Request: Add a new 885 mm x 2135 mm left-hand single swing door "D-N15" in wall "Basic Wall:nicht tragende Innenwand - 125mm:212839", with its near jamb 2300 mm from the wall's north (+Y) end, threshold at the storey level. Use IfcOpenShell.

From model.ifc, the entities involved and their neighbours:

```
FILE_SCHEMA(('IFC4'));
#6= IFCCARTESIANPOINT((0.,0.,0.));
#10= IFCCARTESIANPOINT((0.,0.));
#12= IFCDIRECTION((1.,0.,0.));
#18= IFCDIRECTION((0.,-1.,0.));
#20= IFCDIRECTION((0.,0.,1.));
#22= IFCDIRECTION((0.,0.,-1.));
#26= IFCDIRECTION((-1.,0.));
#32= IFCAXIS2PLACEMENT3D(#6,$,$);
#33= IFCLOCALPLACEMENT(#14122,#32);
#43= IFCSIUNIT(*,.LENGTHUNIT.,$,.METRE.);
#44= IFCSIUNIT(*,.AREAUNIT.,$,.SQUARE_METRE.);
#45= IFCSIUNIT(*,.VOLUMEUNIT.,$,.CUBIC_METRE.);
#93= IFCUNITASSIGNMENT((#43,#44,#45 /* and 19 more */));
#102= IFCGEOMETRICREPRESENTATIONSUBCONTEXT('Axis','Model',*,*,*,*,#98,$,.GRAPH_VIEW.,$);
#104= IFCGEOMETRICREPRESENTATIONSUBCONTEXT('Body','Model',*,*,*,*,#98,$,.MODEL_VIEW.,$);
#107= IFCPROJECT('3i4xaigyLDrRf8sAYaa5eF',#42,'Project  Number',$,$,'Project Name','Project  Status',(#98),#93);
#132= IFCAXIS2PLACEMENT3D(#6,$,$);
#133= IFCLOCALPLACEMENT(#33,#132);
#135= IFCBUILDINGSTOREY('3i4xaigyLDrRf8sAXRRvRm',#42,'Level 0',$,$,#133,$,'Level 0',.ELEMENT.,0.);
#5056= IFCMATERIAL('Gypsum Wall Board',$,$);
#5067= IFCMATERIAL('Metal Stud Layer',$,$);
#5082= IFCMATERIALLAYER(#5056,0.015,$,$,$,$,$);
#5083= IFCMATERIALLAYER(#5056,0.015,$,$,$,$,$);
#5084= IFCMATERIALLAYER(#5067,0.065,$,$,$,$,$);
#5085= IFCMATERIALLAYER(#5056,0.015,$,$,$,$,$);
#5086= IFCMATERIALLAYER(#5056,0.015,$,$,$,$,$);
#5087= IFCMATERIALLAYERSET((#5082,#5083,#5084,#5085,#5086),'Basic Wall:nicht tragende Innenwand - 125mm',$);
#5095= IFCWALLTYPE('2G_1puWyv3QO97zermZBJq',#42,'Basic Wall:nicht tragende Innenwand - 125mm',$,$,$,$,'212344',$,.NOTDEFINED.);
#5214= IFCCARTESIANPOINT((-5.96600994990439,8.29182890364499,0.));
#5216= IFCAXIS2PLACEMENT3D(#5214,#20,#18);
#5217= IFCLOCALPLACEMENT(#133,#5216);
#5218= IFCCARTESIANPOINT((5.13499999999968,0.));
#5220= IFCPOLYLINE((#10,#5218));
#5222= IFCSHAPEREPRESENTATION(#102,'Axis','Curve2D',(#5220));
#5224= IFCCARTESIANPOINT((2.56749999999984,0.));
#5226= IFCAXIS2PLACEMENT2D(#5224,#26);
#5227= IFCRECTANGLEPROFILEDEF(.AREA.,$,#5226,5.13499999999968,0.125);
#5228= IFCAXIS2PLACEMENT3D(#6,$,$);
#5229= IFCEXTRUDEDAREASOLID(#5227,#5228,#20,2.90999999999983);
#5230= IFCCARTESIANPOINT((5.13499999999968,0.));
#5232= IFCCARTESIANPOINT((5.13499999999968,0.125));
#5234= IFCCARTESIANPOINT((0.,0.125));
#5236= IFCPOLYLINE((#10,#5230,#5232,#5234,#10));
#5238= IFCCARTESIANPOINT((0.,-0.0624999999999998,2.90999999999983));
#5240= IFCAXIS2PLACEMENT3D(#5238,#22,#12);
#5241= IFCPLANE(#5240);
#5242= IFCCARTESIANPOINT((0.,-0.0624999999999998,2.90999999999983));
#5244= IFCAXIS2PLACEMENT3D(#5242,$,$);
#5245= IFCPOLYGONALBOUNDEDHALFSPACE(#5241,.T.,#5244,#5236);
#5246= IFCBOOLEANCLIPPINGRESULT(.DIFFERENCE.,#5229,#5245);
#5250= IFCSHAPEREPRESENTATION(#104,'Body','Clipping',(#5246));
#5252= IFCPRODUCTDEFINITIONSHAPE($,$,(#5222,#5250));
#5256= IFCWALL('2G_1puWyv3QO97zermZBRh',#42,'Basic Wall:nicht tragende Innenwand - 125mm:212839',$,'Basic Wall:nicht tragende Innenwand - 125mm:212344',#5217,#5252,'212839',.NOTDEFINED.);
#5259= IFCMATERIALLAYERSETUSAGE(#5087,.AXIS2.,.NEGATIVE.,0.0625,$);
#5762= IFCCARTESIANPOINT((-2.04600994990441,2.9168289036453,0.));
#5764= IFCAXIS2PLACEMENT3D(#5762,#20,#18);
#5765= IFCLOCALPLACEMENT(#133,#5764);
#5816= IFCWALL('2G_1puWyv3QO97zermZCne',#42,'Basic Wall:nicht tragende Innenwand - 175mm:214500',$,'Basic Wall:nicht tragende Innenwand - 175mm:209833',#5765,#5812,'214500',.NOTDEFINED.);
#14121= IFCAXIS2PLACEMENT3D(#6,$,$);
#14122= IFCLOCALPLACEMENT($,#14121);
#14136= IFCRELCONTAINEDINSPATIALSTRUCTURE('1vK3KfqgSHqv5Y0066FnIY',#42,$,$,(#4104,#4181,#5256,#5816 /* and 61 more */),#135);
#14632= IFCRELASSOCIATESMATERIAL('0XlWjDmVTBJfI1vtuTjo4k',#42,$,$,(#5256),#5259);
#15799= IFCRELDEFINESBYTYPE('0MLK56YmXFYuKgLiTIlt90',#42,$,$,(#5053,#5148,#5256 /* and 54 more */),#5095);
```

```python
import numpy as np
import ifcopenshell
import ifcopenshell.api.feature
import ifcopenshell.api.geometry
import ifcopenshell.api.root
import ifcopenshell.api.spatial
import ifcopenshell.geom
import ifcopenshell.util.element
import ifcopenshell.util.placement
import ifcopenshell.util.representation
import ifcopenshell.util.shape
import ifcopenshell.util.unit

model = ifcopenshell.open("model.ifc")
unit_scale = ifcopenshell.util.unit.calculate_unit_scale(model)
settings = ifcopenshell.geom.settings()


def volume(element):
    """Net volume in cubic metres, openings subtracted."""
    shape = ifcopenshell.geom.create_shape(settings, element)
    return ifcopenshell.util.shape.get_volume(shape.geometry)


wall = model.by_guid("2G_1puWyv3QO97zermZBRh")
storey = ifcopenshell.util.element.get_container(wall, ifc_class="IfcBuildingStorey")
context = ifcopenshell.util.representation.get_context(model, "Model", "Body", "MODEL_VIEW")
before = volume(wall)

width, height, from_end, sill = 0.885, 2.135, 2.3, 0.0  # metres

# The wall runs along its own X axis, and the end named is its -X end.
wall_shape = ifcopenshell.geom.create_shape(settings, wall)
x, y, z = ifcopenshell.util.shape.get_vertices(wall_shape.geometry).T
start = x.min() + from_end
face, thickness = float(y.min()), float(y.max() - y.min())
wall_matrix = ifcopenshell.util.placement.get_local_placement(wall.ObjectPlacement)
level = ifcopenshell.util.placement.get_local_placement(storey.ObjectPlacement)[2, 3]


def in_wall(x, y):
    """Placement at x, y metres in the wall's axes, at sill height."""
    matrix = wall_matrix.copy()
    matrix[:, 3] = wall_matrix @ np.array([x / unit_scale, y / unit_scale, 0.0, 1.0])
    matrix[2, 3] = level + sill / unit_scale
    return matrix


# Opening: a box that overshoots both wall faces by 50 mm.
opening = ifcopenshell.api.root.create_entity(model, ifc_class="IfcOpeningElement", predefined_type="OPENING")
box = ifcopenshell.api.geometry.add_wall_representation(
    model, context=context, length=width, height=height, thickness=thickness + 0.1
)
ifcopenshell.api.geometry.assign_representation(model, product=opening, representation=box)
ifcopenshell.api.geometry.edit_object_placement(model, product=opening, matrix=in_wall(start, face - 0.05), is_si=False)
ifcopenshell.api.feature.add_feature(model, feature=opening, element=wall)

door = ifcopenshell.api.root.create_entity(model, ifc_class="IfcDoor", name="D-N15", predefined_type="DOOR")
door.OverallWidth, door.OverallHeight = width / unit_scale, height / unit_scale
door.OperationType = "SINGLE_SWING_LEFT"
body = ifcopenshell.api.geometry.add_door_representation(
    model,
    context=context,
    overall_width=door.OverallWidth,
    overall_height=door.OverallHeight,
    operation_type="SINGLE_SWING_LEFT",
    lining_properties={"LiningDepth": thickness / unit_scale, "ThresholdDepth": thickness / unit_scale},
)
ifcopenshell.api.geometry.assign_representation(model, product=door, representation=body)
ifcopenshell.api.spatial.assign_container(model, products=[door], relating_structure=storey)
ifcopenshell.api.feature.add_filling(model, opening=opening, element=door)

# The lining spans the wall, so the door starts at the wall face.
ifcopenshell.api.geometry.edit_object_placement(model, product=door, matrix=in_wall(start, face), is_si=False)

after = volume(wall)

print(f"wall volume {before:.3f} -> {after:.3f} m3")

model.write("model_updated.ifc")
```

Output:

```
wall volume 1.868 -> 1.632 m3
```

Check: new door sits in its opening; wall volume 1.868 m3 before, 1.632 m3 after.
